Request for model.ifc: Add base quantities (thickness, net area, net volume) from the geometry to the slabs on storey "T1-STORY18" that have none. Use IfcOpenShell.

First a look at what the model holds.

```python
import ifcopenshell
import ifcopenshell.util.element
import ifcopenshell.util.unit

model = ifcopenshell.open("model.ifc")
print(model.schema)
for unit_type in ("LENGTHUNIT", "AREAUNIT", "VOLUMEUNIT"):
    print(unit_type, ifcopenshell.util.unit.calculate_unit_scale(model, unit_type))
storey = next(s for s in model.by_type("IfcBuildingStorey") if s.Name == "T1-STORY18")
slabs = [e for e in ifcopenshell.util.element.get_decomposition(storey) if e.is_a("IfcSlab")]
for e in sorted(slabs, key=lambda e: e.id()):
    print(e.id(), e.is_a(), e.Name, list(ifcopenshell.util.element.get_psets(e, qtos_only=True)), sep=" | ")
```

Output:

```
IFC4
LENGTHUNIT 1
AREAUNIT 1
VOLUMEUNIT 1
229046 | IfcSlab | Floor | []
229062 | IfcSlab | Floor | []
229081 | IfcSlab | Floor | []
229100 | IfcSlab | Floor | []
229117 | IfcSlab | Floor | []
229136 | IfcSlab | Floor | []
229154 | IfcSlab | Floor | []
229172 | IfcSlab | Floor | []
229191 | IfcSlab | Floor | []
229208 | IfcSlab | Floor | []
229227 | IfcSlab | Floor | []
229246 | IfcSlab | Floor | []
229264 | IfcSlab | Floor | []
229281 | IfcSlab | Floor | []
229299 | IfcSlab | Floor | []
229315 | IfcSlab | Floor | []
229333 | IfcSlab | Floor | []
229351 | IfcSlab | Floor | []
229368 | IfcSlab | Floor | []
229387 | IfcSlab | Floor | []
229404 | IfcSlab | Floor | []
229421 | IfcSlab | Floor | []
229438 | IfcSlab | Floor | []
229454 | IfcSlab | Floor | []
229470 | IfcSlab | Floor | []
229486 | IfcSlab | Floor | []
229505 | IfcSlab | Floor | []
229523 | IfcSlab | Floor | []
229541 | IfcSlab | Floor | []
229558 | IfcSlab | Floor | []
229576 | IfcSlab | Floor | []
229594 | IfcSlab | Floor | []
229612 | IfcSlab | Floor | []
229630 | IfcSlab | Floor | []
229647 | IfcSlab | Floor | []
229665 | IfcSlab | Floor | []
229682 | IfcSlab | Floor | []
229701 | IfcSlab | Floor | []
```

```python
import ifcopenshell
import ifcopenshell.api.pset
import ifcopenshell.geom
import ifcopenshell.util.element
import ifcopenshell.util.shape
import ifcopenshell.util.unit

model = ifcopenshell.open("model.ifc")
unit_scale = ifcopenshell.util.unit.calculate_unit_scale(model)
area_scale = ifcopenshell.util.unit.calculate_unit_scale(model, "AREAUNIT")
volume_scale = ifcopenshell.util.unit.calculate_unit_scale(model, "VOLUMEUNIT")
settings = ifcopenshell.geom.settings()

storey = next(s for s in model.by_type("IfcBuildingStorey") if s.Name == "T1-STORY18")
slabs = [e for e in ifcopenshell.util.element.get_decomposition(storey) if e.is_a("IfcSlab")]

for e in sorted(slabs, key=lambda e: e.id()):
    if ifcopenshell.util.element.get_psets(e, qtos_only=True, should_inherit=False):
        continue
    # Geometry comes back in metres, in the element's own axes.
    shape = ifcopenshell.geom.create_shape(settings, e)
    values = {
        "Width": ifcopenshell.util.shape.get_z(shape.geometry) / unit_scale,
        "NetArea": ifcopenshell.util.shape.get_footprint_area(shape.geometry) / area_scale,
        "NetVolume": ifcopenshell.util.shape.get_volume(shape.geometry) / volume_scale,
    }
    qto = ifcopenshell.api.pset.add_qto(model, product=e, name="Qto_SlabBaseQuantities")
    ifcopenshell.api.pset.edit_qto(model, qto=qto, properties=values)
    print(e.id(), {k: round(v, 3) for k, v in values.items()})

model.write("model_v2.ifc")
```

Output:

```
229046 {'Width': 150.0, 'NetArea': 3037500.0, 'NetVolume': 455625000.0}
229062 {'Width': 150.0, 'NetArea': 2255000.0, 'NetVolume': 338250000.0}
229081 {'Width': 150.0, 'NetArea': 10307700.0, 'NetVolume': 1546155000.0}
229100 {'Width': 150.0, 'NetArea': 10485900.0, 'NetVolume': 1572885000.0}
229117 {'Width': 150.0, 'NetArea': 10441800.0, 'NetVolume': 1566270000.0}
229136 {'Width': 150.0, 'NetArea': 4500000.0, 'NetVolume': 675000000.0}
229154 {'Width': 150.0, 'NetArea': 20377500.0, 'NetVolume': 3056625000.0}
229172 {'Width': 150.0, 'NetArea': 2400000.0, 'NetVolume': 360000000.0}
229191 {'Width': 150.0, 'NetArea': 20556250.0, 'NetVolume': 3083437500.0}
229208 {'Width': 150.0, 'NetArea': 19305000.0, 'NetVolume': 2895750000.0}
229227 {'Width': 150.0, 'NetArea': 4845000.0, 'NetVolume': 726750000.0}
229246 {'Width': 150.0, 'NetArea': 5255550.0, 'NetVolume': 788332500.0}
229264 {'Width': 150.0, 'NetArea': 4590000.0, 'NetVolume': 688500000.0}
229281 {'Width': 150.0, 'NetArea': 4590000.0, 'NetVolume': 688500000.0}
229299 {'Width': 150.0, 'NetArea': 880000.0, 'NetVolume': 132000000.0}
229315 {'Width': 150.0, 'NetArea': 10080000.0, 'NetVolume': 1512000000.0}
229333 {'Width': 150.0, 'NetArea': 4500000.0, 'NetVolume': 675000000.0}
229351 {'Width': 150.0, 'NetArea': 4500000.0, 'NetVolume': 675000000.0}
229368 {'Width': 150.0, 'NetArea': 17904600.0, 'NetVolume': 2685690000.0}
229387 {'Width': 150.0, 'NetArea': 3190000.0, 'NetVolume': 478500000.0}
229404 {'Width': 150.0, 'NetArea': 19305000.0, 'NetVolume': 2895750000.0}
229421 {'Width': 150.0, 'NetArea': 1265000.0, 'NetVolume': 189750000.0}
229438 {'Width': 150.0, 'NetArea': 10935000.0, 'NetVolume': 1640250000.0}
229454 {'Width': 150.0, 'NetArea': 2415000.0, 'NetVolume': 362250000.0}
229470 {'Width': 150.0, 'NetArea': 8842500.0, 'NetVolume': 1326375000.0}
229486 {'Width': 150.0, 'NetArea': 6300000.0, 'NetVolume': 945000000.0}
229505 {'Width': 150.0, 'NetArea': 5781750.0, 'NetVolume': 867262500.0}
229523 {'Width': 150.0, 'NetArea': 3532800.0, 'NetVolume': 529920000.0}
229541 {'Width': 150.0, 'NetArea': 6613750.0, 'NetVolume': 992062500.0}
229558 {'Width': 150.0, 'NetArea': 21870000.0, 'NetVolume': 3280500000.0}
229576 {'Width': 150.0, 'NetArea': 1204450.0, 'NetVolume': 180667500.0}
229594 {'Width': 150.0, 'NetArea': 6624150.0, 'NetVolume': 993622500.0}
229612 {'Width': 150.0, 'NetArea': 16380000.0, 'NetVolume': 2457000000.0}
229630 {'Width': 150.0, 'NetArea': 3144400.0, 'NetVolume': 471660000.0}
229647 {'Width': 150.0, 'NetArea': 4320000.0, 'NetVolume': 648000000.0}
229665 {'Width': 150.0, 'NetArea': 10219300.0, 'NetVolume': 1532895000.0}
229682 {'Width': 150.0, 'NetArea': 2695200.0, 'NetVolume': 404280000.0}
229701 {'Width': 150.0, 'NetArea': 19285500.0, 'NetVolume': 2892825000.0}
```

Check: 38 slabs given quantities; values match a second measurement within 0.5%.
